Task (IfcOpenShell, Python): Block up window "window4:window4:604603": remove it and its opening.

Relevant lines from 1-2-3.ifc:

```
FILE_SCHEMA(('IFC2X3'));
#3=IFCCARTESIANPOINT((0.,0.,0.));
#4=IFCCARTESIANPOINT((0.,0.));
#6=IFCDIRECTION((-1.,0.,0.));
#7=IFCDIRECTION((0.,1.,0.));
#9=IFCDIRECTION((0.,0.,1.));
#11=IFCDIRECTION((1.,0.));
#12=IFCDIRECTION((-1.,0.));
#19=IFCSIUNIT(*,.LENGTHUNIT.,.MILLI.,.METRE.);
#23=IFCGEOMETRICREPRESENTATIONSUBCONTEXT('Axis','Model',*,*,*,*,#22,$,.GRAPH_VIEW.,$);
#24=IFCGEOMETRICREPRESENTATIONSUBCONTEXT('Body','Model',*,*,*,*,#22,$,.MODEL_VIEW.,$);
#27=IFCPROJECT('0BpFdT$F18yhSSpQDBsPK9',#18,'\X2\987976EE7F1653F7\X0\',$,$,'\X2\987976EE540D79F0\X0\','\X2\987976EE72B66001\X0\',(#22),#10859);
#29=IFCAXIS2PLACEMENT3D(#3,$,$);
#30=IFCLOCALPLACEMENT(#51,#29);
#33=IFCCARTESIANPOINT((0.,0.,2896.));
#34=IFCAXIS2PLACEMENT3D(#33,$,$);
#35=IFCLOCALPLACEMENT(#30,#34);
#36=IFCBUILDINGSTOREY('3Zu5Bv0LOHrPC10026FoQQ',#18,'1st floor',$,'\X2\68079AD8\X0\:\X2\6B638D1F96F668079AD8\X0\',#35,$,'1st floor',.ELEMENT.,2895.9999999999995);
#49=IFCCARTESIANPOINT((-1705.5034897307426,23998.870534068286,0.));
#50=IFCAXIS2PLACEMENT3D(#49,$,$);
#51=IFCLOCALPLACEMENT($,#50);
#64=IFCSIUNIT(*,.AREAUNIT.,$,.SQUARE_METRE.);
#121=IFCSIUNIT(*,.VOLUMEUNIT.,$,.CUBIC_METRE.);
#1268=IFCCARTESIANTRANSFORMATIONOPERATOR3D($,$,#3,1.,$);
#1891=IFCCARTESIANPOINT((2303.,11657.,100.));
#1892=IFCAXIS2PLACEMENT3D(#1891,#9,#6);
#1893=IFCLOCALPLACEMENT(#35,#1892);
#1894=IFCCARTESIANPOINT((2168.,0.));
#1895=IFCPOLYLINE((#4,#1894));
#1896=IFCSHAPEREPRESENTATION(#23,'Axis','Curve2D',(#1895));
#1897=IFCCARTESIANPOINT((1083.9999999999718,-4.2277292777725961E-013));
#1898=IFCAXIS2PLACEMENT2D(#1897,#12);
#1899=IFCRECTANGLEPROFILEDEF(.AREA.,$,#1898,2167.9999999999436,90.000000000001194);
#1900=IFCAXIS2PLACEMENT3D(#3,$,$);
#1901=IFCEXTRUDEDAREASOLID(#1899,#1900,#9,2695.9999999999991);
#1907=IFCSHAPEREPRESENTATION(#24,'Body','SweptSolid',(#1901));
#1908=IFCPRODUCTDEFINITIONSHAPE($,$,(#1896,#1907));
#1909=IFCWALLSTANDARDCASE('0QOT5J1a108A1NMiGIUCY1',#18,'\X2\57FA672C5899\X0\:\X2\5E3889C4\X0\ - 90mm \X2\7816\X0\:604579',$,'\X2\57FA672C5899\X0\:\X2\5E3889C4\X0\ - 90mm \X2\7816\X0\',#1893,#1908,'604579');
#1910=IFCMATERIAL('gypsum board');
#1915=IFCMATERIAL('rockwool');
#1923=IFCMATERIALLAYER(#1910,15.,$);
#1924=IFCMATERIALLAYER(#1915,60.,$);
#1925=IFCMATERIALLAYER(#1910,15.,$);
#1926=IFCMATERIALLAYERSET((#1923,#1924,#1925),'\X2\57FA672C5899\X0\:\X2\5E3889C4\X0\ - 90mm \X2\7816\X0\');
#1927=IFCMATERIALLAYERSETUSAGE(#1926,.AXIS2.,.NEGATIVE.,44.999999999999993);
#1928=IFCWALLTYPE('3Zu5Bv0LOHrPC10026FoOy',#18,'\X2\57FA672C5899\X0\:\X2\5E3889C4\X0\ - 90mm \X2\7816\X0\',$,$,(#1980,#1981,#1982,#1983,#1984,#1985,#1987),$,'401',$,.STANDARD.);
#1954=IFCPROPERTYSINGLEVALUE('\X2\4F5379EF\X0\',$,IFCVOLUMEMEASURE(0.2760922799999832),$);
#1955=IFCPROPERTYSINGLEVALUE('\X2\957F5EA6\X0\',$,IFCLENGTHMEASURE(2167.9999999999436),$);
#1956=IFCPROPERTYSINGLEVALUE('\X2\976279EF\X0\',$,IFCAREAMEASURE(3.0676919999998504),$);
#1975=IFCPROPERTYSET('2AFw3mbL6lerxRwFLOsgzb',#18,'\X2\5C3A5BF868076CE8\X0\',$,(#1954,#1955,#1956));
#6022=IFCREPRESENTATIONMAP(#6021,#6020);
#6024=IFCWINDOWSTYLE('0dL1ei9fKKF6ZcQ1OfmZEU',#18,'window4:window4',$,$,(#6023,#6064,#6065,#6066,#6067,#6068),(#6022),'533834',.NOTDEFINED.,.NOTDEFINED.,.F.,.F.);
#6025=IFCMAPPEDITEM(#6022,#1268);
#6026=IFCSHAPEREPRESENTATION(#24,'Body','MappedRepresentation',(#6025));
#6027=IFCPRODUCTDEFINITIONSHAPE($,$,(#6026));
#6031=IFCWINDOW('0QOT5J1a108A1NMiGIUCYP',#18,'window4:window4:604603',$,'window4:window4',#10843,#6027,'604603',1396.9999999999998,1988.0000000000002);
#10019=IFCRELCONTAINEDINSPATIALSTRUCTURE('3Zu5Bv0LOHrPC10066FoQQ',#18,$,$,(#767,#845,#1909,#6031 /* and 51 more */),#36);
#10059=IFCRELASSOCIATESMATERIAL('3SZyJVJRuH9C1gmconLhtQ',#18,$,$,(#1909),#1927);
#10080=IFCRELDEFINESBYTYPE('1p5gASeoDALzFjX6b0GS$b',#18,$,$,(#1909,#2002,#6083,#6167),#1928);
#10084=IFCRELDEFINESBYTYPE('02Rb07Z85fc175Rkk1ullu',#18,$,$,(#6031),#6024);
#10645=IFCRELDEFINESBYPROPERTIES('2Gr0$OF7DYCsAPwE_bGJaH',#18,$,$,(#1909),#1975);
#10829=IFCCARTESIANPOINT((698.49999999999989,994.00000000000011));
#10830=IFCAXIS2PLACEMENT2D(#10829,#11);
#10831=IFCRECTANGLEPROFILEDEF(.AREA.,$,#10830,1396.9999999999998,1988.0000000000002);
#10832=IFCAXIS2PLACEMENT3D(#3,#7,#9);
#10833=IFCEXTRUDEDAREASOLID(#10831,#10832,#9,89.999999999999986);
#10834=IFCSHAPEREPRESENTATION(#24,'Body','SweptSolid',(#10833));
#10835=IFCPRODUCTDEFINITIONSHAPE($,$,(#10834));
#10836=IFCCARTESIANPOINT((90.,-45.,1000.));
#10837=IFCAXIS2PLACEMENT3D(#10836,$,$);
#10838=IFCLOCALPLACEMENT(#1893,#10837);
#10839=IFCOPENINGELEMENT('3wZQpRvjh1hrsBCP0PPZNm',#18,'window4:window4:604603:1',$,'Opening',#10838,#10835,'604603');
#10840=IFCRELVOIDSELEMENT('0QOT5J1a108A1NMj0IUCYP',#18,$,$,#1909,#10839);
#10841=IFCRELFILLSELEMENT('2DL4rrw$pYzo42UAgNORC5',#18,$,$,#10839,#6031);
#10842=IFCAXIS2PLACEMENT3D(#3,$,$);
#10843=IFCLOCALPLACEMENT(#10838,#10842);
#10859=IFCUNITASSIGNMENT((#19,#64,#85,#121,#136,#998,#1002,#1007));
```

```python
import ifcopenshell
import ifcopenshell.api.feature
import ifcopenshell.api.pset
import ifcopenshell.api.root
import ifcopenshell.geom
import ifcopenshell.util.element
import ifcopenshell.util.shape
import ifcopenshell.util.unit

model = ifcopenshell.open("1-2-3.ifc")
area_scale = ifcopenshell.util.unit.calculate_unit_scale(model, "AREAUNIT")
volume_scale = ifcopenshell.util.unit.calculate_unit_scale(model, "VOLUMEUNIT")
settings = ifcopenshell.geom.settings()


def volume(element):
    """Net volume in cubic metres, openings subtracted."""
    shape = ifcopenshell.geom.create_shape(settings, element)
    return ifcopenshell.util.shape.get_volume(shape.geometry)


window = model.by_guid("0QOT5J1a108A1NMiGIUCYP")
opening = window.FillsVoids[0].RelatingOpeningElement
wall = opening.VoidsElements[0].RelatingBuildingElement
before = volume(wall)

ifcopenshell.api.root.remove_product(model, product=window)
ifcopenshell.api.feature.remove_feature(model, feature=opening)

after = volume(wall)
thickness = 0.09  # wall thickness in metres

# Update the wall's stored quantities.
pset = model.by_id(ifcopenshell.util.element.get_pset(wall, "尺寸标注", should_inherit=False)["id"])
ifcopenshell.api.pset.edit_pset(model, pset=pset, properties={
    "体积": model.create_entity("IfcVolumeMeasure", after / volume_scale),
    "面积": model.create_entity("IfcAreaMeasure", after / thickness / area_scale),
})

print(f"wall volume {before:.3f} -> {after:.3f} m3")

model.write("1-2-3_updated.ifc")
```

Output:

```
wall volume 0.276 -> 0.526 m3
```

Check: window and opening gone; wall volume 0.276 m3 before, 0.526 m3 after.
